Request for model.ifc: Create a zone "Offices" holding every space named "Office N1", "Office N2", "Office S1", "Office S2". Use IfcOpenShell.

First a look at what the model holds.

```python
import ifcopenshell

model = ifcopenshell.open("model.ifc")
print(model.schema)
seen = {}
for space in model.by_type("IfcSpace"):
    seen[space.LongName] = seen.get(space.LongName, 0) + 1
for name, count in sorted(seen.items(), key=str):
    print(count, "x", name)
print("zones:", [z.Name for z in model.by_type("IfcZone")][:20])
```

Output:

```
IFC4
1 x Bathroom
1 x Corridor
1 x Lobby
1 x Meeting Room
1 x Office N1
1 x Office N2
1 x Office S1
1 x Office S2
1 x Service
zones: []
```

```python
import ifcopenshell
import ifcopenshell.api.group
import ifcopenshell.api.root

model = ifcopenshell.open("model.ifc")

names = {"Office N1", "Office N2", "Office S1", "Office S2"}
spaces = [s for s in model.by_type("IfcSpace") if s.LongName in names]

zone = ifcopenshell.api.root.create_entity(model, ifc_class="IfcZone", name="Offices")
ifcopenshell.api.group.assign_group(model, products=spaces, group=zone)
print(len(spaces), "spaces in", zone.Name)

model.write("model_rev.ifc")
```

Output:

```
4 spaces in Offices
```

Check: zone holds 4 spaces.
